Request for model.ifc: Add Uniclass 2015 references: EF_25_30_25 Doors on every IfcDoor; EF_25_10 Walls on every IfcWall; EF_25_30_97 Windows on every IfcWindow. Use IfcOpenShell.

First a look at what the model holds.

```python
import ifcopenshell

model = ifcopenshell.open("model.ifc")
print(model.schema)
print("classifications:", [c.Name for c in model.by_type("IfcClassification")])
for ifc_class in ("IfcDoor", "IfcRoof", "IfcStair", "IfcWall", "IfcWindow"):
    print(ifc_class, len(model.by_type(ifc_class)))
```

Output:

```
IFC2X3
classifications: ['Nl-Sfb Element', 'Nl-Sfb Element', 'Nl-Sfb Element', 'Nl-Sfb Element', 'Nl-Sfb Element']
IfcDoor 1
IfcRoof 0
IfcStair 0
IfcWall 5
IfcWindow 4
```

```python
import ifcopenshell
import ifcopenshell.api.classification

model = ifcopenshell.open("model.ifc")

# IFC2X3 requires Source and Edition and has no link from the project to the system.
system = model.create_entity("IfcClassification", Source="NBS", Edition="2015", Name="Uniclass 2015")

codes = {
    "IfcDoor": ("EF_25_30_25", "Doors"),
    "IfcWall": ("EF_25_10", "Walls"),
    "IfcWindow": ("EF_25_30_97", "Windows"),
}
for ifc_class, (code, name) in codes.items():
    products = model.by_type(ifc_class)
    ifcopenshell.api.classification.add_reference(
        model, products=products, classification=system, identification=code, name=name
    )
    print(code, len(products))

model.write("model_rev.ifc")
```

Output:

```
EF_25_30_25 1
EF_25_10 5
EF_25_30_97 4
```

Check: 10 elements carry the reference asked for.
